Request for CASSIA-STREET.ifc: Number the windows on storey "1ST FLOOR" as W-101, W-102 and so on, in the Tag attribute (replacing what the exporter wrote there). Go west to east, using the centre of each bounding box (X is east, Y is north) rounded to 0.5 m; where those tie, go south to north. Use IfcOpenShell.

First a look at what the model holds.

```python
import ifcopenshell
import ifcopenshell.util.element
import ifcopenshell.util.placement

model = ifcopenshell.open("CASSIA-STREET.ifc")
print(model.schema)
storey = next(s for s in model.by_type("IfcBuildingStorey") if s.Name == "1ST FLOOR")
windows = [e for e in ifcopenshell.util.element.get_decomposition(storey) if e.is_a("IfcWindow")]
for e in sorted(windows, key=lambda e: e.id()):
    origin = ifcopenshell.util.placement.get_local_placement(e.ObjectPlacement)[:3, 3]
    print(e.id(), e.Tag, e.Name, origin.round(2) + 0.0, sep=" | ")
```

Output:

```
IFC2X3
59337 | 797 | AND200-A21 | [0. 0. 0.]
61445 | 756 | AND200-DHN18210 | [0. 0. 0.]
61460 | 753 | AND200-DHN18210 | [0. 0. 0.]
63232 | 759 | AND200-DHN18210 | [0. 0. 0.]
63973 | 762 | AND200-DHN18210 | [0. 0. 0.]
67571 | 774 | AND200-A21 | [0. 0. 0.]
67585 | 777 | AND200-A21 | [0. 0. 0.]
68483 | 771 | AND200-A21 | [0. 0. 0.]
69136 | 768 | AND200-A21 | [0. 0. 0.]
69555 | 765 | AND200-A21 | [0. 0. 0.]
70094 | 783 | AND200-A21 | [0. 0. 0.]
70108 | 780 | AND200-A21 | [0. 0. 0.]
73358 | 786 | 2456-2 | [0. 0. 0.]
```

```python
import ifcopenshell
import ifcopenshell.geom
import ifcopenshell.util.element
import ifcopenshell.util.shape

model = ifcopenshell.open("CASSIA-STREET.ifc")
settings = ifcopenshell.geom.settings()
settings.set("use-world-coords", True)


def centre(element):
    shape = ifcopenshell.geom.create_shape(settings, element)
    return ifcopenshell.util.shape.get_bbox_centroid(shape.geometry)


storey = next(s for s in model.by_type("IfcBuildingStorey") if s.Name == "1ST FLOOR")
windows = [e for e in ifcopenshell.util.element.get_decomposition(storey) if e.is_a("IfcWindow")]

# Insertion points can sit at a corner or the storey origin, so sort by the geometry (in metres).
centres = {e: centre(e) for e in windows}
windows.sort(key=lambda e: (round(centres[e][0] / 0.5), centres[e][1]))

for i, e in enumerate(windows, start=1):
    number = f"W-1{i:02d}"
    e.Tag = number
    print(e.id(), number)

model.write("CASSIA-STREET_rev.ifc")
```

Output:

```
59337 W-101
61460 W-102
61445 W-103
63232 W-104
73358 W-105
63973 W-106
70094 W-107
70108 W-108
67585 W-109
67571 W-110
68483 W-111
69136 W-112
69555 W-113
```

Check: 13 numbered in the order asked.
